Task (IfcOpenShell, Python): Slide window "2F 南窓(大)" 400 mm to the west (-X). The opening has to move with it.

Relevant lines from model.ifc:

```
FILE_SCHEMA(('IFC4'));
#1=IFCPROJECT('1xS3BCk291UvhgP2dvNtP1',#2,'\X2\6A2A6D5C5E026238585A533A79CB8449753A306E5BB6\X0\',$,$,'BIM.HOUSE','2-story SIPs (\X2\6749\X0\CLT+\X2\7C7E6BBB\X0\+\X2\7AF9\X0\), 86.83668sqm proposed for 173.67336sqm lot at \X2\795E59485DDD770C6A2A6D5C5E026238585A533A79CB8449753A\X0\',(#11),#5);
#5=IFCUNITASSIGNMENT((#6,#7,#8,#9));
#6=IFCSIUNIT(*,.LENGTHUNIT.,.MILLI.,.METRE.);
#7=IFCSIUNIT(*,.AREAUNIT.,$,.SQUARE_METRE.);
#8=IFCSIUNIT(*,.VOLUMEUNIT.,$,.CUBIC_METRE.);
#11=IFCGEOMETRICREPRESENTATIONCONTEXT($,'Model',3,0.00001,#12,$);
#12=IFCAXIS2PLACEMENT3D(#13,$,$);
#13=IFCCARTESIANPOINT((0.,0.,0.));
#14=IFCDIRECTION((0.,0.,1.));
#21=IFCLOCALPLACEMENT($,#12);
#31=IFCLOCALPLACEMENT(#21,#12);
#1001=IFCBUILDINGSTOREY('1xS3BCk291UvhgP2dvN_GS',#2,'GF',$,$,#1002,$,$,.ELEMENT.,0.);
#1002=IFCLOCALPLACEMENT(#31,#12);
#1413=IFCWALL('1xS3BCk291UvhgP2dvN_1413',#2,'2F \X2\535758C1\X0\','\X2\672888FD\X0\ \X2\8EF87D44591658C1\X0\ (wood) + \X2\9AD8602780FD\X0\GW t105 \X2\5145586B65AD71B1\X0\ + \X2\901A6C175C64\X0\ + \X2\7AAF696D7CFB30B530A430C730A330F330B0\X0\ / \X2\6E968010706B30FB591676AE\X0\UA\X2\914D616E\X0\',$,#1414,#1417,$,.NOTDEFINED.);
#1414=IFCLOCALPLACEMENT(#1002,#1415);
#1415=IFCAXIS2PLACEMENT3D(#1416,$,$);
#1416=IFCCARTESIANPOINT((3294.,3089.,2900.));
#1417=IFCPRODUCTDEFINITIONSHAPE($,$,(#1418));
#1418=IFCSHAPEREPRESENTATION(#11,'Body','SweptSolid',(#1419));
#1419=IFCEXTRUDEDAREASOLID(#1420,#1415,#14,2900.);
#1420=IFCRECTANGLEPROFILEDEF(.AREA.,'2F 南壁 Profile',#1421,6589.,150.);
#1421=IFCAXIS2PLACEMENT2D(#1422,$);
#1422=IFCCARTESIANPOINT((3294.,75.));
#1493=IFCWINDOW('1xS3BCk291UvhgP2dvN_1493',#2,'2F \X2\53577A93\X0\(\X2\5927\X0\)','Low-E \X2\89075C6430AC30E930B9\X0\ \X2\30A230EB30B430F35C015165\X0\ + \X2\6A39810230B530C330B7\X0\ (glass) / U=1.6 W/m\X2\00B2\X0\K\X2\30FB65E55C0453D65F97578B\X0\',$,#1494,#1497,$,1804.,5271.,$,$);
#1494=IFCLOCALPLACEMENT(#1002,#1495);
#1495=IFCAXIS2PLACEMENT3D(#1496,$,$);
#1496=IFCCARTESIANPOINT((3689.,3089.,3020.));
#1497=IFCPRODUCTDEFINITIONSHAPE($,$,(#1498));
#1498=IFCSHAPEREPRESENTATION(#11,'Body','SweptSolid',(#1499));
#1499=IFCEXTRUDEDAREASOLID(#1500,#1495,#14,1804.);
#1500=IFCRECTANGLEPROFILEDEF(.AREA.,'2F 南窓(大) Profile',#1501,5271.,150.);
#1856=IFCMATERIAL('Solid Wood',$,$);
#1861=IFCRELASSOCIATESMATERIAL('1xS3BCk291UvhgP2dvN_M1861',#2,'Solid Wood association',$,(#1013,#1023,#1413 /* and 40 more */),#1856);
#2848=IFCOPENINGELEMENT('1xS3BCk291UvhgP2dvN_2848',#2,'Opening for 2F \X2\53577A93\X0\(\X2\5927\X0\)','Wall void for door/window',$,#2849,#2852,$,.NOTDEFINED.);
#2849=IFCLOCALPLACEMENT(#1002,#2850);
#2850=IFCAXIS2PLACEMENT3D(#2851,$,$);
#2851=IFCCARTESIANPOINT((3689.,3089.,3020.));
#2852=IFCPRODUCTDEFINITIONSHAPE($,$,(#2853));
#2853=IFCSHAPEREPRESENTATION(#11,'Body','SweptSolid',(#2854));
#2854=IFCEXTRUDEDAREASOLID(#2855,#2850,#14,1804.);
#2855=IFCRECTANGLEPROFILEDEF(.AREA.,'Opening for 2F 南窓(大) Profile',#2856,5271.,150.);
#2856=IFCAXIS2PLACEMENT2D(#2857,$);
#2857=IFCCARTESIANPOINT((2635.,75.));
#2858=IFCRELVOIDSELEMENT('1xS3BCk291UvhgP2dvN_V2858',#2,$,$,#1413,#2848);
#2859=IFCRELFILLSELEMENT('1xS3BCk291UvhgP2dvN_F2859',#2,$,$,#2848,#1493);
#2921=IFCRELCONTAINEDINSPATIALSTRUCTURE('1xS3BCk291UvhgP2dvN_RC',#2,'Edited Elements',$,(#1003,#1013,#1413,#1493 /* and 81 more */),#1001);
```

```python
import ifcopenshell
import ifcopenshell.api.geometry
import ifcopenshell.util.placement

model = ifcopenshell.open("model.ifc")

window = model.by_guid("1xS3BCk291UvhgP2dvN_1493")
opening = window.FillsVoids[0].RelatingOpeningElement
wall = opening.VoidsElements[0].RelatingBuildingElement

wall_matrix = ifcopenshell.util.placement.get_local_placement(wall.ObjectPlacement)
shift = wall_matrix[:3, 0] * -400.0
before = ifcopenshell.util.placement.get_local_placement(window.ObjectPlacement)[:3, 3].copy()

# The window is not placed relative to its opening, so move both.
for product in (opening, window):
    matrix = ifcopenshell.util.placement.get_local_placement(product.ObjectPlacement)
    matrix[:3, 3] += shift
    ifcopenshell.api.geometry.edit_object_placement(model, product=product, matrix=matrix, is_si=False)

after = ifcopenshell.util.placement.get_local_placement(window.ObjectPlacement)[:3, 3]
print("window moved by", (after - before).round(3) + 0.0)

model.write("model_rev.ifc")
```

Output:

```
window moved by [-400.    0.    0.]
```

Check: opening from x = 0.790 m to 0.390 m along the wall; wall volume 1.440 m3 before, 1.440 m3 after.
